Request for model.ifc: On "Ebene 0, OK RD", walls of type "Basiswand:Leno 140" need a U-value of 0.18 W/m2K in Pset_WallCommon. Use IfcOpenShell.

First a look at what the model holds.

```python
import ifcopenshell
import ifcopenshell.util.element

model = ifcopenshell.open("model.ifc")
print(model.schema)
storey = next(s for s in model.by_type("IfcBuildingStorey") if s.Name == "Ebene 0, OK RD")
walls = [e for e in ifcopenshell.util.element.get_decomposition(storey) if e.is_a("IfcWall")]
seen = {}
for e in walls:
    element_type = ifcopenshell.util.element.get_type(e)
    key = (element_type.Name if element_type != e and element_type else None, ifcopenshell.util.element.get_pset(e, "Pset_WallCommon", "ThermalTransmittance"))
    seen[key] = seen.get(key, 0) + 1
for (name, value), count in sorted(seen.items(), key=str):
    print(count, "x", name, "|", value)
```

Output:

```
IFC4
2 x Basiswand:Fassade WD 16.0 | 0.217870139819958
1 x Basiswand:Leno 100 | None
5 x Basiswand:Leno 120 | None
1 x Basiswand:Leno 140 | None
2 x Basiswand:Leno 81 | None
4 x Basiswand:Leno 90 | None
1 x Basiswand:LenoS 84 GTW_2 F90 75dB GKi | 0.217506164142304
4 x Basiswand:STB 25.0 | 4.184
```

```python
import ifcopenshell
import ifcopenshell.api.pset
import ifcopenshell.util.element

model = ifcopenshell.open("model.ifc")

storey = next(s for s in model.by_type("IfcBuildingStorey") if s.Name == "Ebene 0, OK RD")
walls = [e for e in ifcopenshell.util.element.get_decomposition(storey) if e.is_a("IfcWall")]

count = 0
for e in walls:
    element_type = ifcopenshell.util.element.get_type(e)
    if element_type in (None, e) or element_type.Name != "Basiswand:Leno 140":
        continue
    # add_pset returns the element's existing set when there is one.
    pset = ifcopenshell.api.pset.add_pset(model, product=e, name="Pset_WallCommon")
    ifcopenshell.api.pset.edit_pset(model, pset=pset, properties={"ThermalTransmittance": 0.18})
    count += 1

print(count, "walls updated")

model.write("model-out.ifc")
```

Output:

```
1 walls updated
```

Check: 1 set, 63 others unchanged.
